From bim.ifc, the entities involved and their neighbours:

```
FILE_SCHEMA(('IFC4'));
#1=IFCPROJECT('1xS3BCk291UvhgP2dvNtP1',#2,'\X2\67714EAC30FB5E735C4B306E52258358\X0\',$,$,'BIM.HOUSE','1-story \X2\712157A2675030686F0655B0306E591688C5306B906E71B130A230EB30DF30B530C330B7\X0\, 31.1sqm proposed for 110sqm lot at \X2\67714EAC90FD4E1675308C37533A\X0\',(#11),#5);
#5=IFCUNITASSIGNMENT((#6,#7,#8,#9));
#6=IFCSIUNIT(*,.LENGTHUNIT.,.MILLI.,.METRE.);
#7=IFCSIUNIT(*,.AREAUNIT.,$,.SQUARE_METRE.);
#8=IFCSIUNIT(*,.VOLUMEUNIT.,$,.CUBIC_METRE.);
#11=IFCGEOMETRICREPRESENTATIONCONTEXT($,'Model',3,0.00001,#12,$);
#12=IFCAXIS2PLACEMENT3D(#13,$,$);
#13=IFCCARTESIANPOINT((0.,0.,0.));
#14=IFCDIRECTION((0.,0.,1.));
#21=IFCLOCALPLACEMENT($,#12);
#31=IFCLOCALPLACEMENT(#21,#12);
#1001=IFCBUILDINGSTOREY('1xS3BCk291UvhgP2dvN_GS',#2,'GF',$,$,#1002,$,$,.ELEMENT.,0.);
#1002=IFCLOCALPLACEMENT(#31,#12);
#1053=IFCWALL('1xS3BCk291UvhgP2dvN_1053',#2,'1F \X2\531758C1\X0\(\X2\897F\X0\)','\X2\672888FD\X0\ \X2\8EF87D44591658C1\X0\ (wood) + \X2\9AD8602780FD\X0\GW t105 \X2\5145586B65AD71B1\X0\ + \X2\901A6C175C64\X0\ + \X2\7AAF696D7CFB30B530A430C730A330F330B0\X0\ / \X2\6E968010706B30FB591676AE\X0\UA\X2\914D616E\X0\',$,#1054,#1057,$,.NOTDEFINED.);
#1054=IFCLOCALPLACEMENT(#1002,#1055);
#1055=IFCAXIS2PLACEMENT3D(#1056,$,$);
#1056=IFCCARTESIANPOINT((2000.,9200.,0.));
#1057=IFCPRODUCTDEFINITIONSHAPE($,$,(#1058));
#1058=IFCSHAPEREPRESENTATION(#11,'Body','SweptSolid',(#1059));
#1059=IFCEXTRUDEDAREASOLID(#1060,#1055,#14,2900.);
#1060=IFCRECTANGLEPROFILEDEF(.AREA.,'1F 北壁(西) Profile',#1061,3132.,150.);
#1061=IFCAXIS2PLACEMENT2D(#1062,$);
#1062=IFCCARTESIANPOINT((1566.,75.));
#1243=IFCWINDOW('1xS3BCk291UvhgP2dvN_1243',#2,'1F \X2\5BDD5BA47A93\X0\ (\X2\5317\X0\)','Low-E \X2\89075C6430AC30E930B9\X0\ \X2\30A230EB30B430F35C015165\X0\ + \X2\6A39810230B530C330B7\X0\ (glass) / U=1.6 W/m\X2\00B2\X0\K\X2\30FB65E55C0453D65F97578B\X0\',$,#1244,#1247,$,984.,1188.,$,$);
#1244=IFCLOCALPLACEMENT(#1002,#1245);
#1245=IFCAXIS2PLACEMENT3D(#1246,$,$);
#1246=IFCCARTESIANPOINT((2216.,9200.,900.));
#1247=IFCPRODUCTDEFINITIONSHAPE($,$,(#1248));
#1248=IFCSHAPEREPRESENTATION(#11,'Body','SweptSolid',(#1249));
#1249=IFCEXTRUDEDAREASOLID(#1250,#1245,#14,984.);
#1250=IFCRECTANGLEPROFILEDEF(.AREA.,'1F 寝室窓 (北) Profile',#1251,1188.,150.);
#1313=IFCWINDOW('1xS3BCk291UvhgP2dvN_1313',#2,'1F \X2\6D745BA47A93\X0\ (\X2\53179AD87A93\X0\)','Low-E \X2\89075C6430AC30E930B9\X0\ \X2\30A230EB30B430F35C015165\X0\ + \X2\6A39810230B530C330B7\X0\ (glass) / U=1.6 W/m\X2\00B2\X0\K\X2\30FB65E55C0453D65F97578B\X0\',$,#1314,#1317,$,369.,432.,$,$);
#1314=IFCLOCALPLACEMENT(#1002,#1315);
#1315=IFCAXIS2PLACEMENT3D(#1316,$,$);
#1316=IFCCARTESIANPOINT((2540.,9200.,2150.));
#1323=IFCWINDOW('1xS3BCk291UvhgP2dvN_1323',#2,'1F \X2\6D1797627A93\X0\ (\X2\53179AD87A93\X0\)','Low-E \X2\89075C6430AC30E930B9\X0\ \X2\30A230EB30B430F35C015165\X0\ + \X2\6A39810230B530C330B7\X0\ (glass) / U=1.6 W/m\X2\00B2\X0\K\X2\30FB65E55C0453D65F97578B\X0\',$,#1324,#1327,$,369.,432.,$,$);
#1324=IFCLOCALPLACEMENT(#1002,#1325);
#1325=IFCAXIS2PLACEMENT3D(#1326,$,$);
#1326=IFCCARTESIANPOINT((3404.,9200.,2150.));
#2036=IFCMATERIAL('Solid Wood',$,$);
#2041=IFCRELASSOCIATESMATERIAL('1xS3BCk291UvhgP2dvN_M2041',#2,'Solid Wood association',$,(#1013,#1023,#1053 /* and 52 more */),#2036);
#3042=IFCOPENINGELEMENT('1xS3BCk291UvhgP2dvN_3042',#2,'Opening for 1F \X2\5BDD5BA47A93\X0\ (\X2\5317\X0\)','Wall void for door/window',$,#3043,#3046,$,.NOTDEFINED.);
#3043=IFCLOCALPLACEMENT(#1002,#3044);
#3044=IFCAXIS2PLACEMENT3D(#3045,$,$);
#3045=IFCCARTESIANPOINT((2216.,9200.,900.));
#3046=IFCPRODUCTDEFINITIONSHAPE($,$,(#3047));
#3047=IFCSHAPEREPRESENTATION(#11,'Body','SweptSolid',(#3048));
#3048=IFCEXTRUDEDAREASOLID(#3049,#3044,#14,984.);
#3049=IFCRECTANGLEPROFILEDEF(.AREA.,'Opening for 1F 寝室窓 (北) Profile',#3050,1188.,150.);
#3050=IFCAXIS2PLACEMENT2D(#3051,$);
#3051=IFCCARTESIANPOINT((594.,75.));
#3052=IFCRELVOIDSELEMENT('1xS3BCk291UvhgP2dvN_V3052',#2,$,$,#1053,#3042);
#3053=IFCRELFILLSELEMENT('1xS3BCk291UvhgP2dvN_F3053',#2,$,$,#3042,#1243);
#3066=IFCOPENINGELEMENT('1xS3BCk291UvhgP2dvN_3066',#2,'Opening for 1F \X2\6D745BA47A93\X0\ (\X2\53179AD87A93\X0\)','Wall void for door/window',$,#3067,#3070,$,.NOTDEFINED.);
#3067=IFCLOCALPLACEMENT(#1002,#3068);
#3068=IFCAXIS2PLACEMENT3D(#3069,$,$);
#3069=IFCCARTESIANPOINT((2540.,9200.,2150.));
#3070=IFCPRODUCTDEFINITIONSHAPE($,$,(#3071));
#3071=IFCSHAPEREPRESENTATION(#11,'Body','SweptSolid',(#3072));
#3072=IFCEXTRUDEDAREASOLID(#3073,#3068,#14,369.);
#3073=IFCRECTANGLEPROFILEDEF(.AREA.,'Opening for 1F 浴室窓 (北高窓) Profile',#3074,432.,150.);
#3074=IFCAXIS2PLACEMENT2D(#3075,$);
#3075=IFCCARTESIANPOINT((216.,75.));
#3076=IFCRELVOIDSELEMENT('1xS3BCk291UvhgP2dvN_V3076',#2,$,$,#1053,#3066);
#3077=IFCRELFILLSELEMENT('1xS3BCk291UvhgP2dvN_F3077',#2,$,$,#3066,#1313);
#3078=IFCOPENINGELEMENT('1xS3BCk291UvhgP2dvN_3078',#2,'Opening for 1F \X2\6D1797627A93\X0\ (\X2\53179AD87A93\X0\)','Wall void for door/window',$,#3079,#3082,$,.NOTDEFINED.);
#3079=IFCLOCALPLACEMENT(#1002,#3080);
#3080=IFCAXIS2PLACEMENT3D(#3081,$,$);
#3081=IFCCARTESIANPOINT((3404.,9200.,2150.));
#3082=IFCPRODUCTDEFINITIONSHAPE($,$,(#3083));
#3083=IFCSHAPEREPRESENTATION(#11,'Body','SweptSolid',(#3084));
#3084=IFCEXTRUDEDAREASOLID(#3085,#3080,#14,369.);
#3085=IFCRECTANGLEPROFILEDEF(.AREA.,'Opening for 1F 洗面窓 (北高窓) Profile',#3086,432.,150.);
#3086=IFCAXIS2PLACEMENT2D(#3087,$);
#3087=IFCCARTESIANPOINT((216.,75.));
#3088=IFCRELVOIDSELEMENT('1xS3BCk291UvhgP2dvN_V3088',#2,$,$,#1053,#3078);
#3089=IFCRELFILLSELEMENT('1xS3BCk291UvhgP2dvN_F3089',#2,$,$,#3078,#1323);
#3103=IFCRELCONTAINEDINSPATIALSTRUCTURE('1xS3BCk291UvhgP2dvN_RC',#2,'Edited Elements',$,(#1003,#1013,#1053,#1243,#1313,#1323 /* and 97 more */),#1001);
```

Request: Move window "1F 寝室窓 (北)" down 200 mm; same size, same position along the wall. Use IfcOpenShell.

```python
import numpy as np
import ifcopenshell
import ifcopenshell.api.geometry
import ifcopenshell.util.placement
import ifcopenshell.util.unit

model = ifcopenshell.open("bim.ifc")
unit_scale = ifcopenshell.util.unit.calculate_unit_scale(model)

window = model.by_guid("1xS3BCk291UvhgP2dvN_1243")
opening = window.FillsVoids[0].RelatingOpeningElement
dz = -0.2 / unit_scale

shift = np.array([0.0, 0.0, dz])
# The window is not placed relative to its opening, so move both.
for product in (opening, window):
    matrix = ifcopenshell.util.placement.get_local_placement(product.ObjectPlacement)
    matrix[:3, 3] += shift
    ifcopenshell.api.geometry.edit_object_placement(model, product=product, matrix=matrix, is_si=False)

print(f"moved by {dz * unit_scale:+.3f} m")

model.write("bim_rev.ifc")
```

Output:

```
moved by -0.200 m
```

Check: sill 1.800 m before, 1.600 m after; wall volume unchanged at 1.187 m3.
